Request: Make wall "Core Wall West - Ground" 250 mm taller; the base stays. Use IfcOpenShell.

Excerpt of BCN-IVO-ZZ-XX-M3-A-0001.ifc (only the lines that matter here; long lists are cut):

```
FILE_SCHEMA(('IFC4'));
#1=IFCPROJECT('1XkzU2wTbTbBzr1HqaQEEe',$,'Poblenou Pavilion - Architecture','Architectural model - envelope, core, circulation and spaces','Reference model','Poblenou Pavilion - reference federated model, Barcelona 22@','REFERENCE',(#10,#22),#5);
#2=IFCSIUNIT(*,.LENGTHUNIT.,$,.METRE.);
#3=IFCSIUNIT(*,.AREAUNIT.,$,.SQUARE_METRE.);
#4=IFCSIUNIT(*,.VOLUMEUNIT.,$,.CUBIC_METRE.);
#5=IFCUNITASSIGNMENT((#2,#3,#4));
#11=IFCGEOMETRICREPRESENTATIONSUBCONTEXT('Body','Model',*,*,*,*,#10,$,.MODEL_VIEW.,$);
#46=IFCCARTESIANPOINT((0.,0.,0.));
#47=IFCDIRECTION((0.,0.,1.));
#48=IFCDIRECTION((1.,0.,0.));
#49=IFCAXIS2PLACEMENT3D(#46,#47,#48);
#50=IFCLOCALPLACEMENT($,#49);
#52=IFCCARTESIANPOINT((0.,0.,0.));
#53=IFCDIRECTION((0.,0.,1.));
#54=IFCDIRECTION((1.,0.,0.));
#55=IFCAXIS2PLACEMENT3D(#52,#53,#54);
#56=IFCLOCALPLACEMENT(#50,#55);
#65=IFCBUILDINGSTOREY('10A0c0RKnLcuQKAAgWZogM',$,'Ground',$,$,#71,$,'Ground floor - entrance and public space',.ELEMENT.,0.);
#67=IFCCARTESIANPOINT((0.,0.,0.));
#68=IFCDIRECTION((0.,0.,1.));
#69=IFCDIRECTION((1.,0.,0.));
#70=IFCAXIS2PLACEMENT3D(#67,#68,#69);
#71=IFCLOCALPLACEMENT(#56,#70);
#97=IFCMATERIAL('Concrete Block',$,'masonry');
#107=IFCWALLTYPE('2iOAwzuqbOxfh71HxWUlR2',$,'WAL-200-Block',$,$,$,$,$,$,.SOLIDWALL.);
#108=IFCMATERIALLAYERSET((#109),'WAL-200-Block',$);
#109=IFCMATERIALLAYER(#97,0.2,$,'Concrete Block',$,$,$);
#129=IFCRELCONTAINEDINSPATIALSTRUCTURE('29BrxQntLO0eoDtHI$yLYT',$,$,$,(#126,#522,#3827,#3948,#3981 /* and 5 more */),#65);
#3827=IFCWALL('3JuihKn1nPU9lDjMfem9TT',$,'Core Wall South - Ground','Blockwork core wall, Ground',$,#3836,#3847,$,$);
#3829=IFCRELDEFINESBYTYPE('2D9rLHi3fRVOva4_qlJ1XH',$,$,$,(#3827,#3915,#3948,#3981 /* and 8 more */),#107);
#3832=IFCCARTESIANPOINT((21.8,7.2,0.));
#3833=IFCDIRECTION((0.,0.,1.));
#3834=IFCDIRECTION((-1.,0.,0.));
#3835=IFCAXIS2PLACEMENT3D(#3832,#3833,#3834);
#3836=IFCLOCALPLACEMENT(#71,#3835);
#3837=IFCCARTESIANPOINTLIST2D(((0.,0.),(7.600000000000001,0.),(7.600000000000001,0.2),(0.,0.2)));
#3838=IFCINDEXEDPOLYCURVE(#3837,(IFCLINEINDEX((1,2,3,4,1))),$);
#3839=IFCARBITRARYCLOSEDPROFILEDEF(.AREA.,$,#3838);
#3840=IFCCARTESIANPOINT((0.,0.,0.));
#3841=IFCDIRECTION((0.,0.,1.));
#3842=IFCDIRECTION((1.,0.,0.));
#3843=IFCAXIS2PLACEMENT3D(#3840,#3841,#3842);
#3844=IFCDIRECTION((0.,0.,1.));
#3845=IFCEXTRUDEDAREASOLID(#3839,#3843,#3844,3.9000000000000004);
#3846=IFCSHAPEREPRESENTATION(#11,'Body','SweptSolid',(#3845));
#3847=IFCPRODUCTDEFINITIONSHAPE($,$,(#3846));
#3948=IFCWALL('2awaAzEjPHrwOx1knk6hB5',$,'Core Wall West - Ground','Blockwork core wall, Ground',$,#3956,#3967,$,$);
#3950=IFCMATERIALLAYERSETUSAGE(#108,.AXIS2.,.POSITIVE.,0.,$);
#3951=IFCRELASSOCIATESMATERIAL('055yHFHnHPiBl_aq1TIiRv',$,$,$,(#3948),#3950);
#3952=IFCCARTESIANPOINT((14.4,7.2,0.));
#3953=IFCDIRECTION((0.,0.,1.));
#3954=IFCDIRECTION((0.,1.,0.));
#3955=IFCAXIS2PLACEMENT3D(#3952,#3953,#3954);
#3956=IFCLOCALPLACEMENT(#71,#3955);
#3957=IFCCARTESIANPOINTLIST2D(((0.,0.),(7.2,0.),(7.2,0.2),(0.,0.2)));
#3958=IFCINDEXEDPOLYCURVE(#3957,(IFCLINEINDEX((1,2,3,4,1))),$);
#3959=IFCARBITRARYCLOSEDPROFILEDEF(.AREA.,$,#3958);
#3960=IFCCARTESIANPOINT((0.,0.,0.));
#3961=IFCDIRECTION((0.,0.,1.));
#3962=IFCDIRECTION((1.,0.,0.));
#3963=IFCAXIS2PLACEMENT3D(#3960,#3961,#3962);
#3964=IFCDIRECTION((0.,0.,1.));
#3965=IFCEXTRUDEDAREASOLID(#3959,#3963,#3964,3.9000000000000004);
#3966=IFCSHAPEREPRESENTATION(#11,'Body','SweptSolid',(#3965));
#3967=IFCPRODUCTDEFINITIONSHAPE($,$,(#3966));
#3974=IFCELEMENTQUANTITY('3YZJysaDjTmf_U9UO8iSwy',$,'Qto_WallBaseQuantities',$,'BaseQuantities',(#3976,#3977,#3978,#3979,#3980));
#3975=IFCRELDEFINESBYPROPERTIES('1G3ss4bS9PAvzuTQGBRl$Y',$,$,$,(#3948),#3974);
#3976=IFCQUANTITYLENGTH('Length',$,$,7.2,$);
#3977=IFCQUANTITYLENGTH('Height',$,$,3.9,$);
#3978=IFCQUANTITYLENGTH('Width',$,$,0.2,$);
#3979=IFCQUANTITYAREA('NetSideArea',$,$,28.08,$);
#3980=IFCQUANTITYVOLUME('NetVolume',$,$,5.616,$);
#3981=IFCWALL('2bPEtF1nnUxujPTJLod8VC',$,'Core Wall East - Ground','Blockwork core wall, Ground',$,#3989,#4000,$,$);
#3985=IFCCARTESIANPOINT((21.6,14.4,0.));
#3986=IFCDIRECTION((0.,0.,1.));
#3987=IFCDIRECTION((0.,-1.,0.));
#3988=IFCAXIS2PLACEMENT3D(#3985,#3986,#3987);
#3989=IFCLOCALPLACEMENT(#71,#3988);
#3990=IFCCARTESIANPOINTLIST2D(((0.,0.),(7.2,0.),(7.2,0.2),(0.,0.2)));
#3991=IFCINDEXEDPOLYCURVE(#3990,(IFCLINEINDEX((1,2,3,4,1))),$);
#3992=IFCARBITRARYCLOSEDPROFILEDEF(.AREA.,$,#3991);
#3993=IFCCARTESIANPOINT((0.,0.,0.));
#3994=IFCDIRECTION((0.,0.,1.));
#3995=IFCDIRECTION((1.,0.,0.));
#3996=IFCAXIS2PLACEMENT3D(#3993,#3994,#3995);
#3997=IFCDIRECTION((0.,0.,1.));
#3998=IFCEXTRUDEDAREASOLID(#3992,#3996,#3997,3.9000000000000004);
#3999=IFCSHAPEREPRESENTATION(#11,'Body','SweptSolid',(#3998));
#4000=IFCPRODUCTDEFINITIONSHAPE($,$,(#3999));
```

```python
import ifcopenshell
import ifcopenshell.api.pset
import ifcopenshell.geom
import ifcopenshell.util.element
import ifcopenshell.util.representation
import ifcopenshell.util.shape
import ifcopenshell.util.unit

model = ifcopenshell.open("BCN-IVO-ZZ-XX-M3-A-0001.ifc")
unit_scale = ifcopenshell.util.unit.calculate_unit_scale(model)
area_scale = ifcopenshell.util.unit.calculate_unit_scale(model, "AREAUNIT")
volume_scale = ifcopenshell.util.unit.calculate_unit_scale(model, "VOLUMEUNIT")
settings = ifcopenshell.geom.settings()


def volume(element):
    """Net volume in cubic metres, openings subtracted."""
    shape = ifcopenshell.geom.create_shape(settings, element)
    return ifcopenshell.util.shape.get_volume(shape.geometry)


wall = model.by_guid("2awaAzEjPHrwOx1knk6hB5")
before = volume(wall)

body = ifcopenshell.util.representation.get_representation(wall, "Model", "Body")
solid = body.Items[0]
old_height = solid.Depth
solid.Depth += 0.25 / unit_scale
after = volume(wall)
thickness = 0.2  # wall thickness in metres

# Update the stored height, areas and volumes.
qto = model.by_id(ifcopenshell.util.element.get_pset(wall, "Qto_WallBaseQuantities", should_inherit=False)["id"])
ifcopenshell.api.pset.edit_qto(model, qto=qto, properties={
    "Height": solid.Depth,
    "NetSideArea": after / thickness / area_scale,
    "NetVolume": after / volume_scale,
})

print(f"height {old_height:g} -> {solid.Depth:g}, volume {before:.3f} -> {after:.3f} m3")

model.write("BCN-IVO-ZZ-XX-M3-A-0001_v2.ifc")
```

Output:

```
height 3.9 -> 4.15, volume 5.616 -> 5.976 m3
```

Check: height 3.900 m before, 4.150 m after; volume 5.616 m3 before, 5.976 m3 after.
